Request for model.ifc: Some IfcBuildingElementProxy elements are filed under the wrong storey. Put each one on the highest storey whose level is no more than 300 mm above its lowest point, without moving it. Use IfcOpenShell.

First a look at what the model holds.

```python
import ifcopenshell
import ifcopenshell.util.element
import ifcopenshell.util.placement

model = ifcopenshell.open("model.ifc")
print(model.schema)
for storey in model.by_type("IfcBuildingStorey"):
    level = ifcopenshell.util.placement.get_storey_elevation(storey)
    count = sum(e.is_a("IfcBuildingElementProxy") for e in ifcopenshell.util.element.get_contained(storey))
    print(storey.id(), storey.Name, round(level, 3), count, sep=" | ")
```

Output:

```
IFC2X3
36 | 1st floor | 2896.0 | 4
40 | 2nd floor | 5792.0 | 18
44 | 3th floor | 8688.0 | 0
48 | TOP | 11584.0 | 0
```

```python
import ifcopenshell
import ifcopenshell.api.spatial
import ifcopenshell.geom
import ifcopenshell.util.element
import ifcopenshell.util.placement
import ifcopenshell.util.shape
import ifcopenshell.util.unit

model = ifcopenshell.open("model.ifc")
unit_scale = ifcopenshell.util.unit.calculate_unit_scale(model)
settings = ifcopenshell.geom.settings()

levels = sorted(
    ((ifcopenshell.util.placement.get_storey_elevation(s) * unit_scale, s) for s in model.by_type("IfcBuildingStorey")),
    key=lambda pair: pair[0],
)

for e in model.by_type("IfcBuildingElementProxy"):
    current = e.ContainedInStructure[0].RelatingStructure if e.ContainedInStructure else None
    if current is None or not current.is_a("IfcBuildingStorey"):
        continue
    shape = ifcopenshell.geom.create_shape(settings, e)
    bottom = ifcopenshell.util.shape.get_shape_bottom_elevation(shape, shape.geometry)
    below = [s for level, s in levels if level <= bottom + 0.3]
    storey = below[-1] if below else levels[0][1]
    if storey != current:
        # assign_container keeps the world position.
        ifcopenshell.api.spatial.assign_container(model, products=[e], relating_structure=storey)
        print(e.id(), current.Name, "->", storey.Name)

model.write("model_edited.ifc")
```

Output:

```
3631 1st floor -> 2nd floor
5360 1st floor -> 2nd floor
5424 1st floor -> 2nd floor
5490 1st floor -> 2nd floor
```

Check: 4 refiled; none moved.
